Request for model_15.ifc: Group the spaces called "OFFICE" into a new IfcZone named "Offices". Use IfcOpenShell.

First a look at what the model holds.

```python
import ifcopenshell

model = ifcopenshell.open("model_15.ifc")
print(model.schema)
seen = {}
for space in model.by_type("IfcSpace"):
    seen[space.LongName] = seen.get(space.LongName, 0) + 1
for name, count in sorted(seen.items(), key=str):
    print(count, "x", name)
print("zones:", [z.Name for z in model.by_type("IfcZone")][:20])
```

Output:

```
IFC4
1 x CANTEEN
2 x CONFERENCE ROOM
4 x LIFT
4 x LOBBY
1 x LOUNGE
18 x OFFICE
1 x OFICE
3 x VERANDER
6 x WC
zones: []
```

```python
import ifcopenshell
import ifcopenshell.api.group
import ifcopenshell.api.root

model = ifcopenshell.open("model_15.ifc")

names = {"OFFICE"}
spaces = [s for s in model.by_type("IfcSpace") if s.LongName in names]

zone = ifcopenshell.api.root.create_entity(model, ifc_class="IfcZone", name="Offices")
ifcopenshell.api.group.assign_group(model, products=spaces, group=zone)
print(len(spaces), "spaces in", zone.Name)

model.write("model_15_edited.ifc")
```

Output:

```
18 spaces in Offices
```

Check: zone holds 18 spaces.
